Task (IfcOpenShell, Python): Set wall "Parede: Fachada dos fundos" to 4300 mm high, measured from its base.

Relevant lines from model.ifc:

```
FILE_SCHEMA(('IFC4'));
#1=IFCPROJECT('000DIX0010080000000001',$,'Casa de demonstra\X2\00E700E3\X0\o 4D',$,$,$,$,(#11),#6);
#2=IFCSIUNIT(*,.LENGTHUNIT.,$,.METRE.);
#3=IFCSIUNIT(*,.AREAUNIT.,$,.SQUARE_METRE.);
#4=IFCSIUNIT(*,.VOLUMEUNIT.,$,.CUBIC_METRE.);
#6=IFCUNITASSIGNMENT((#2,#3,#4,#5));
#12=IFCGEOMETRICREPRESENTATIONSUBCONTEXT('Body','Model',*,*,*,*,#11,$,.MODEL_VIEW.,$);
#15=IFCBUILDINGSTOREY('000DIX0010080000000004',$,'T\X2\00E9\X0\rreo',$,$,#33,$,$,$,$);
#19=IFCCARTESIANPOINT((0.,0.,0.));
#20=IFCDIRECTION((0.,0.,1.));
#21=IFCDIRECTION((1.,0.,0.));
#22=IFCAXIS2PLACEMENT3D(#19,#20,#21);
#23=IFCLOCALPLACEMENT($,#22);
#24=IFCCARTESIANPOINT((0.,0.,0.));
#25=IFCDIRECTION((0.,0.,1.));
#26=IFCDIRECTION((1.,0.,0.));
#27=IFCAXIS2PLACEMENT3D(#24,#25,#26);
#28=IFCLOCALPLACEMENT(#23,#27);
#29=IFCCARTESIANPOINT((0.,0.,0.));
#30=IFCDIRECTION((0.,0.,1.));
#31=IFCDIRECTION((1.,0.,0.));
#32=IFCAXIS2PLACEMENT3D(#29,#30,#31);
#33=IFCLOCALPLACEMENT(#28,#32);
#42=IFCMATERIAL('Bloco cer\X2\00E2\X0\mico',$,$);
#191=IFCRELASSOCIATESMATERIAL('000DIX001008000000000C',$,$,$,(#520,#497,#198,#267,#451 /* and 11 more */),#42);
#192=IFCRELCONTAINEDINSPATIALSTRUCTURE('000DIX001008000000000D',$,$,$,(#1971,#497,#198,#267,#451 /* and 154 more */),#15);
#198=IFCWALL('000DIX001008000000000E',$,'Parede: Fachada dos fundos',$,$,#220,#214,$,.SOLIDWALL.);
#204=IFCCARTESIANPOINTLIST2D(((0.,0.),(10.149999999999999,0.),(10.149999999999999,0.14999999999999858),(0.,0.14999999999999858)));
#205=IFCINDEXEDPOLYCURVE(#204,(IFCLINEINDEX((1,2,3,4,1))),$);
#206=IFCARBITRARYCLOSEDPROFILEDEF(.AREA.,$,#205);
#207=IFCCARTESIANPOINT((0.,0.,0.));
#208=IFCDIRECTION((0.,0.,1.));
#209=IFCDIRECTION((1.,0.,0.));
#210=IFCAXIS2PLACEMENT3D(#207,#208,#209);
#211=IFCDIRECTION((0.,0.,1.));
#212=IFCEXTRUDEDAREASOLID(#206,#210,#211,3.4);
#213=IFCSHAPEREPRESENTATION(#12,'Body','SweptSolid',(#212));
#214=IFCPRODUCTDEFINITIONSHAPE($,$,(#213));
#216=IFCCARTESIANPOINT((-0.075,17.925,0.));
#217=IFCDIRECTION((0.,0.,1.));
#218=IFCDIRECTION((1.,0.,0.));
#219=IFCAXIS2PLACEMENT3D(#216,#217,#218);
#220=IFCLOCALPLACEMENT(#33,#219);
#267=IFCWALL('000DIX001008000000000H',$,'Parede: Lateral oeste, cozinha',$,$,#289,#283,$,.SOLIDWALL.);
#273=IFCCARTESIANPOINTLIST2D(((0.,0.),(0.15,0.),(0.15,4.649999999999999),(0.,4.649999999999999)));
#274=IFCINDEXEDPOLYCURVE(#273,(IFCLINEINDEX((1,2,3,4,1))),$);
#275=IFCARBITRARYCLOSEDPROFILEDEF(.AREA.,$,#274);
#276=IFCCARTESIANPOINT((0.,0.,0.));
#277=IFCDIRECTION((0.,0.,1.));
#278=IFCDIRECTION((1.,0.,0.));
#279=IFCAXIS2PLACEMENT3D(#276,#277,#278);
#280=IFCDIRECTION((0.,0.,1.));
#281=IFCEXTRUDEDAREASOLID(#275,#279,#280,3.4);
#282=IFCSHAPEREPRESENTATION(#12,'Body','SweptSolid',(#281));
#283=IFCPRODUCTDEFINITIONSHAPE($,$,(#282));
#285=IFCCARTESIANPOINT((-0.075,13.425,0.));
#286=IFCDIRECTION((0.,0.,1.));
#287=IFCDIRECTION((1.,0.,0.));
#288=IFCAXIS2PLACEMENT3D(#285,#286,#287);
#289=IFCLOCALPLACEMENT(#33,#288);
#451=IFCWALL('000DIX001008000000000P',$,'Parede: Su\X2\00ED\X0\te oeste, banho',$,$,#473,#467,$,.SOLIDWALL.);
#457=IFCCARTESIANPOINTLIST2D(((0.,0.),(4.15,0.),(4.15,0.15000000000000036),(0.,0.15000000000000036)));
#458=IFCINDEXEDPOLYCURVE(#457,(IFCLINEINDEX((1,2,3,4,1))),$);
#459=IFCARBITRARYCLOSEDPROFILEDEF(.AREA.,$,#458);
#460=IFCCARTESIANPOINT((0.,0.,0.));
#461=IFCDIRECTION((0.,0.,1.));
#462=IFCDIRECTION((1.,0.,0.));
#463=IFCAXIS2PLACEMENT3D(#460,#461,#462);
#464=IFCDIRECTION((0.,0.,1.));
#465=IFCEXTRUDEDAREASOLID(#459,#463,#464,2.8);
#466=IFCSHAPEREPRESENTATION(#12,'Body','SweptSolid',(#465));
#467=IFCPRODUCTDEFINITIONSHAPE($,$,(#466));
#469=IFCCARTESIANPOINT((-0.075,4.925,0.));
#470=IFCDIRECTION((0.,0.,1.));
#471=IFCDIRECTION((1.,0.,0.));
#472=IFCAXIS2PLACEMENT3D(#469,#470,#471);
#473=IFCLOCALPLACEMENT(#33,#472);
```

```python
import ifcopenshell
import ifcopenshell.geom
import ifcopenshell.util.representation
import ifcopenshell.util.shape

model = ifcopenshell.open("model.ifc")
settings = ifcopenshell.geom.settings()


def volume(element):
    """Net volume in cubic metres, openings subtracted."""
    shape = ifcopenshell.geom.create_shape(settings, element)
    return ifcopenshell.util.shape.get_volume(shape.geometry)


wall = model.by_guid("000DIX001008000000000E")
before = volume(wall)

body = ifcopenshell.util.representation.get_representation(wall, "Model", "Body")
solid = body.Items[0]
old_height = solid.Depth
solid.Depth = 4.3
after = volume(wall)

print(f"height {old_height:g} -> {solid.Depth:g}, volume {before:.3f} -> {after:.3f} m3")

model.write("model_updated.ifc")
```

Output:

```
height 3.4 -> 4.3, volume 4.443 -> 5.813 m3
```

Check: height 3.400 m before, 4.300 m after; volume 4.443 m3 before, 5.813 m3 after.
